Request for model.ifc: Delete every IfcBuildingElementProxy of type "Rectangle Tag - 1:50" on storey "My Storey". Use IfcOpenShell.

First a look at what the model holds.

```python
import ifcopenshell
import ifcopenshell.util.element

model = ifcopenshell.open("model.ifc")
print(model.schema)
storey = next(s for s in model.by_type("IfcBuildingStorey") if s.Name == "My Storey")
proxies = [e for e in ifcopenshell.util.element.get_decomposition(storey) if e.is_a("IfcBuildingElementProxy")]
seen = {}
for e in proxies:
    element_type = ifcopenshell.util.element.get_type(e)
    name = element_type.Name if element_type not in (None, e) else None
    seen[name] = seen.get(name, 0) + 1
for name, count in sorted(seen.items(), key=str):
    print(count, "x", name)
```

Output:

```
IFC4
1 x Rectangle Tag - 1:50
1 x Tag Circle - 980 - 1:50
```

```python
import ifcopenshell
import ifcopenshell.api.root
import ifcopenshell.util.element

model = ifcopenshell.open("model.ifc")

storey = next(s for s in model.by_type("IfcBuildingStorey") if s.Name == "My Storey")
proxies = [e for e in ifcopenshell.util.element.get_decomposition(storey) if e.is_a("IfcBuildingElementProxy")]
targets = [e for e in proxies if (t := ifcopenshell.util.element.get_type(e)) not in (None, e) and t.Name == "Rectangle Tag - 1:50"]

for e in targets:
    ifcopenshell.api.root.remove_product(model, product=e)
print(len(targets), "removed")

model.write("model_rev.ifc")
```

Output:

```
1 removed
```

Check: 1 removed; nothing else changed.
